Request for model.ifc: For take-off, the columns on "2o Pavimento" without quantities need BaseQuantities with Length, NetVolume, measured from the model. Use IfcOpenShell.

First a look at what the model holds.

```python
import ifcopenshell
import ifcopenshell.util.element
import ifcopenshell.util.unit

model = ifcopenshell.open("model.ifc")
print(model.schema)
for unit_type in ("LENGTHUNIT", "AREAUNIT", "VOLUMEUNIT"):
    print(unit_type, ifcopenshell.util.unit.calculate_unit_scale(model, unit_type))
storey = next(s for s in model.by_type("IfcBuildingStorey") if s.Name == "2o Pavimento")
columns = [e for e in ifcopenshell.util.element.get_decomposition(storey) if e.is_a("IfcColumn")]
for e in sorted(columns, key=lambda e: e.id()):
    print(e.id(), e.is_a(), e.Name, list(ifcopenshell.util.element.get_psets(e, qtos_only=True)), sep=" | ")
```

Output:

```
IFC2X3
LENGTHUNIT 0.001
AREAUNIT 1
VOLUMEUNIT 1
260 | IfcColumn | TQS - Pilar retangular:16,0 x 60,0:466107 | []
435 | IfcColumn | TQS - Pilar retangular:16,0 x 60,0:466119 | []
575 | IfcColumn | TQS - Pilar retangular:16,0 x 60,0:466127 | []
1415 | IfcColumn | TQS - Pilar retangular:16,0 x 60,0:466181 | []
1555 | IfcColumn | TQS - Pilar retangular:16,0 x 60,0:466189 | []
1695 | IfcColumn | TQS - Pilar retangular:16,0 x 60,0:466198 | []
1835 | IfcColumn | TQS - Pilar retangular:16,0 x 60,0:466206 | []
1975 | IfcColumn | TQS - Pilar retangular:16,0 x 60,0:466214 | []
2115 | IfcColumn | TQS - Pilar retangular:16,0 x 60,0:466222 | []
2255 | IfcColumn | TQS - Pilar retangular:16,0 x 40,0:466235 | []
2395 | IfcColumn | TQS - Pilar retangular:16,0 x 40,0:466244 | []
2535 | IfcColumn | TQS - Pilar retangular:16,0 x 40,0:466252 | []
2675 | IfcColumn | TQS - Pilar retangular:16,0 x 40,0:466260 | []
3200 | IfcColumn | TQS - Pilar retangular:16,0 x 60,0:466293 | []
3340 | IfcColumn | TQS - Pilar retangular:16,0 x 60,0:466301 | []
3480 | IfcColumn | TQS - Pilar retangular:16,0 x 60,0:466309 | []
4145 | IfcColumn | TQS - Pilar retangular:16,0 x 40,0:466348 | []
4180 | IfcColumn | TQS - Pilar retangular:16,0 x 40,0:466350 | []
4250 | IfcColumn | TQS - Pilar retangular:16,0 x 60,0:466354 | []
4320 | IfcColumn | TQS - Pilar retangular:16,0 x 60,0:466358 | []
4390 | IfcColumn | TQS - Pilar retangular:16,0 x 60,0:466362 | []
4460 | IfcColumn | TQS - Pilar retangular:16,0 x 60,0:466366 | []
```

```python
import ifcopenshell
import ifcopenshell.api.pset
import ifcopenshell.geom
import ifcopenshell.util.element
import ifcopenshell.util.shape
import ifcopenshell.util.unit

model = ifcopenshell.open("model.ifc")
unit_scale = ifcopenshell.util.unit.calculate_unit_scale(model)
volume_scale = ifcopenshell.util.unit.calculate_unit_scale(model, "VOLUMEUNIT")
settings = ifcopenshell.geom.settings()

storey = next(s for s in model.by_type("IfcBuildingStorey") if s.Name == "2o Pavimento")
columns = [e for e in ifcopenshell.util.element.get_decomposition(storey) if e.is_a("IfcColumn")]

for e in sorted(columns, key=lambda e: e.id()):
    if ifcopenshell.util.element.get_psets(e, qtos_only=True, should_inherit=False):
        continue
    # Geometry comes back in metres, in the element's own axes.
    shape = ifcopenshell.geom.create_shape(settings, e)
    values = {
        "Length": ifcopenshell.util.shape.get_z(shape.geometry) / unit_scale,
        "NetVolume": ifcopenshell.util.shape.get_volume(shape.geometry) / volume_scale,
    }
    qto = ifcopenshell.api.pset.add_qto(model, product=e, name="BaseQuantities")
    ifcopenshell.api.pset.edit_qto(model, qto=qto, properties=values)
    print(e.id(), {k: round(v, 3) for k, v in values.items()})

model.write("model_rev.ifc")
```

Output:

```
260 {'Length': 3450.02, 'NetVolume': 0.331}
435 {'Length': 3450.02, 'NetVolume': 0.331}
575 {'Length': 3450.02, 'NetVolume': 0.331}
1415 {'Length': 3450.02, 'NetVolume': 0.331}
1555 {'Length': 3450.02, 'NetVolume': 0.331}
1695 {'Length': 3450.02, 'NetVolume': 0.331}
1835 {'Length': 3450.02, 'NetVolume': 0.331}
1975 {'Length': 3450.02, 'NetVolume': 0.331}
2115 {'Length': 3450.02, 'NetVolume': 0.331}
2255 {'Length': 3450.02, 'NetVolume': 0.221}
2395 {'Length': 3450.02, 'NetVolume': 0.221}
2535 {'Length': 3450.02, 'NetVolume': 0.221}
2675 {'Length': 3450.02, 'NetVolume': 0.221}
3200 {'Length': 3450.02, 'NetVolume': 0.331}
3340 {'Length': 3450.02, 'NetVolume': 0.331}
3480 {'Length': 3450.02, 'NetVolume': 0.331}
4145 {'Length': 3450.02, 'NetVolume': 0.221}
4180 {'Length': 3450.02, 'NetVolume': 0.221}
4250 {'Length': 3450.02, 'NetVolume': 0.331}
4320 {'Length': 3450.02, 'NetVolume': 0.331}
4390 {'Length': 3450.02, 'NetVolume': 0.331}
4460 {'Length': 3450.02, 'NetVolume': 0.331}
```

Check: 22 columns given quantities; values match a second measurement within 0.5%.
